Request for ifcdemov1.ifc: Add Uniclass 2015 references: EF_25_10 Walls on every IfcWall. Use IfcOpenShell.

First a look at what the model holds.

```python
import ifcopenshell

model = ifcopenshell.open("ifcdemov1.ifc")
print(model.schema)
print("classifications:", [c.Name for c in model.by_type("IfcClassification")])
for ifc_class in ("IfcDoor", "IfcRoof", "IfcStair", "IfcWall", "IfcWindow"):
    print(ifc_class, len(model.by_type(ifc_class)))
```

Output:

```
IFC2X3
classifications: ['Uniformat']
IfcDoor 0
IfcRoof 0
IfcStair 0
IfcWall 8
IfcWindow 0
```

```python
import ifcopenshell
import ifcopenshell.api.classification

model = ifcopenshell.open("ifcdemov1.ifc")

# IFC2X3 requires Source and Edition and has no link from the project to the system.
system = model.create_entity("IfcClassification", Source="NBS", Edition="2015", Name="Uniclass 2015")

codes = {
    "IfcWall": ("EF_25_10", "Walls"),
}
for ifc_class, (code, name) in codes.items():
    products = model.by_type(ifc_class)
    ifcopenshell.api.classification.add_reference(
        model, products=products, classification=system, identification=code, name=name
    )
    print(code, len(products))

model.write("ifcdemov1_updated.ifc")
```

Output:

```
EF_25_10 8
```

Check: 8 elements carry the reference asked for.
